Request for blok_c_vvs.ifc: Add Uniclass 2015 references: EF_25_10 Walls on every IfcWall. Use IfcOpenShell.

First a look at what the model holds.

```python
import ifcopenshell

model = ifcopenshell.open("blok_c_vvs.ifc")
print(model.schema)
print("classifications:", [c.Name for c in model.by_type("IfcClassification")])
for ifc_class in ("IfcDoor", "IfcRoof", "IfcStair", "IfcWall", "IfcWindow"):
    print(ifc_class, len(model.by_type(ifc_class)))
```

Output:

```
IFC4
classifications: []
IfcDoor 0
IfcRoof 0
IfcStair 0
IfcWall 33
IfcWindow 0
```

```python
import ifcopenshell
import ifcopenshell.api.classification

model = ifcopenshell.open("blok_c_vvs.ifc")

system = ifcopenshell.api.classification.add_classification(model, classification="Uniclass 2015")

codes = {
    "IfcWall": ("EF_25_10", "Walls"),
}
for ifc_class, (code, name) in codes.items():
    products = model.by_type(ifc_class)
    ifcopenshell.api.classification.add_reference(
        model, products=products, classification=system, identification=code, name=name
    )
    print(code, len(products))

model.write("blok_c_vvs_edited.ifc")
```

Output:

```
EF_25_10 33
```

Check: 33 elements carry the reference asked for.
